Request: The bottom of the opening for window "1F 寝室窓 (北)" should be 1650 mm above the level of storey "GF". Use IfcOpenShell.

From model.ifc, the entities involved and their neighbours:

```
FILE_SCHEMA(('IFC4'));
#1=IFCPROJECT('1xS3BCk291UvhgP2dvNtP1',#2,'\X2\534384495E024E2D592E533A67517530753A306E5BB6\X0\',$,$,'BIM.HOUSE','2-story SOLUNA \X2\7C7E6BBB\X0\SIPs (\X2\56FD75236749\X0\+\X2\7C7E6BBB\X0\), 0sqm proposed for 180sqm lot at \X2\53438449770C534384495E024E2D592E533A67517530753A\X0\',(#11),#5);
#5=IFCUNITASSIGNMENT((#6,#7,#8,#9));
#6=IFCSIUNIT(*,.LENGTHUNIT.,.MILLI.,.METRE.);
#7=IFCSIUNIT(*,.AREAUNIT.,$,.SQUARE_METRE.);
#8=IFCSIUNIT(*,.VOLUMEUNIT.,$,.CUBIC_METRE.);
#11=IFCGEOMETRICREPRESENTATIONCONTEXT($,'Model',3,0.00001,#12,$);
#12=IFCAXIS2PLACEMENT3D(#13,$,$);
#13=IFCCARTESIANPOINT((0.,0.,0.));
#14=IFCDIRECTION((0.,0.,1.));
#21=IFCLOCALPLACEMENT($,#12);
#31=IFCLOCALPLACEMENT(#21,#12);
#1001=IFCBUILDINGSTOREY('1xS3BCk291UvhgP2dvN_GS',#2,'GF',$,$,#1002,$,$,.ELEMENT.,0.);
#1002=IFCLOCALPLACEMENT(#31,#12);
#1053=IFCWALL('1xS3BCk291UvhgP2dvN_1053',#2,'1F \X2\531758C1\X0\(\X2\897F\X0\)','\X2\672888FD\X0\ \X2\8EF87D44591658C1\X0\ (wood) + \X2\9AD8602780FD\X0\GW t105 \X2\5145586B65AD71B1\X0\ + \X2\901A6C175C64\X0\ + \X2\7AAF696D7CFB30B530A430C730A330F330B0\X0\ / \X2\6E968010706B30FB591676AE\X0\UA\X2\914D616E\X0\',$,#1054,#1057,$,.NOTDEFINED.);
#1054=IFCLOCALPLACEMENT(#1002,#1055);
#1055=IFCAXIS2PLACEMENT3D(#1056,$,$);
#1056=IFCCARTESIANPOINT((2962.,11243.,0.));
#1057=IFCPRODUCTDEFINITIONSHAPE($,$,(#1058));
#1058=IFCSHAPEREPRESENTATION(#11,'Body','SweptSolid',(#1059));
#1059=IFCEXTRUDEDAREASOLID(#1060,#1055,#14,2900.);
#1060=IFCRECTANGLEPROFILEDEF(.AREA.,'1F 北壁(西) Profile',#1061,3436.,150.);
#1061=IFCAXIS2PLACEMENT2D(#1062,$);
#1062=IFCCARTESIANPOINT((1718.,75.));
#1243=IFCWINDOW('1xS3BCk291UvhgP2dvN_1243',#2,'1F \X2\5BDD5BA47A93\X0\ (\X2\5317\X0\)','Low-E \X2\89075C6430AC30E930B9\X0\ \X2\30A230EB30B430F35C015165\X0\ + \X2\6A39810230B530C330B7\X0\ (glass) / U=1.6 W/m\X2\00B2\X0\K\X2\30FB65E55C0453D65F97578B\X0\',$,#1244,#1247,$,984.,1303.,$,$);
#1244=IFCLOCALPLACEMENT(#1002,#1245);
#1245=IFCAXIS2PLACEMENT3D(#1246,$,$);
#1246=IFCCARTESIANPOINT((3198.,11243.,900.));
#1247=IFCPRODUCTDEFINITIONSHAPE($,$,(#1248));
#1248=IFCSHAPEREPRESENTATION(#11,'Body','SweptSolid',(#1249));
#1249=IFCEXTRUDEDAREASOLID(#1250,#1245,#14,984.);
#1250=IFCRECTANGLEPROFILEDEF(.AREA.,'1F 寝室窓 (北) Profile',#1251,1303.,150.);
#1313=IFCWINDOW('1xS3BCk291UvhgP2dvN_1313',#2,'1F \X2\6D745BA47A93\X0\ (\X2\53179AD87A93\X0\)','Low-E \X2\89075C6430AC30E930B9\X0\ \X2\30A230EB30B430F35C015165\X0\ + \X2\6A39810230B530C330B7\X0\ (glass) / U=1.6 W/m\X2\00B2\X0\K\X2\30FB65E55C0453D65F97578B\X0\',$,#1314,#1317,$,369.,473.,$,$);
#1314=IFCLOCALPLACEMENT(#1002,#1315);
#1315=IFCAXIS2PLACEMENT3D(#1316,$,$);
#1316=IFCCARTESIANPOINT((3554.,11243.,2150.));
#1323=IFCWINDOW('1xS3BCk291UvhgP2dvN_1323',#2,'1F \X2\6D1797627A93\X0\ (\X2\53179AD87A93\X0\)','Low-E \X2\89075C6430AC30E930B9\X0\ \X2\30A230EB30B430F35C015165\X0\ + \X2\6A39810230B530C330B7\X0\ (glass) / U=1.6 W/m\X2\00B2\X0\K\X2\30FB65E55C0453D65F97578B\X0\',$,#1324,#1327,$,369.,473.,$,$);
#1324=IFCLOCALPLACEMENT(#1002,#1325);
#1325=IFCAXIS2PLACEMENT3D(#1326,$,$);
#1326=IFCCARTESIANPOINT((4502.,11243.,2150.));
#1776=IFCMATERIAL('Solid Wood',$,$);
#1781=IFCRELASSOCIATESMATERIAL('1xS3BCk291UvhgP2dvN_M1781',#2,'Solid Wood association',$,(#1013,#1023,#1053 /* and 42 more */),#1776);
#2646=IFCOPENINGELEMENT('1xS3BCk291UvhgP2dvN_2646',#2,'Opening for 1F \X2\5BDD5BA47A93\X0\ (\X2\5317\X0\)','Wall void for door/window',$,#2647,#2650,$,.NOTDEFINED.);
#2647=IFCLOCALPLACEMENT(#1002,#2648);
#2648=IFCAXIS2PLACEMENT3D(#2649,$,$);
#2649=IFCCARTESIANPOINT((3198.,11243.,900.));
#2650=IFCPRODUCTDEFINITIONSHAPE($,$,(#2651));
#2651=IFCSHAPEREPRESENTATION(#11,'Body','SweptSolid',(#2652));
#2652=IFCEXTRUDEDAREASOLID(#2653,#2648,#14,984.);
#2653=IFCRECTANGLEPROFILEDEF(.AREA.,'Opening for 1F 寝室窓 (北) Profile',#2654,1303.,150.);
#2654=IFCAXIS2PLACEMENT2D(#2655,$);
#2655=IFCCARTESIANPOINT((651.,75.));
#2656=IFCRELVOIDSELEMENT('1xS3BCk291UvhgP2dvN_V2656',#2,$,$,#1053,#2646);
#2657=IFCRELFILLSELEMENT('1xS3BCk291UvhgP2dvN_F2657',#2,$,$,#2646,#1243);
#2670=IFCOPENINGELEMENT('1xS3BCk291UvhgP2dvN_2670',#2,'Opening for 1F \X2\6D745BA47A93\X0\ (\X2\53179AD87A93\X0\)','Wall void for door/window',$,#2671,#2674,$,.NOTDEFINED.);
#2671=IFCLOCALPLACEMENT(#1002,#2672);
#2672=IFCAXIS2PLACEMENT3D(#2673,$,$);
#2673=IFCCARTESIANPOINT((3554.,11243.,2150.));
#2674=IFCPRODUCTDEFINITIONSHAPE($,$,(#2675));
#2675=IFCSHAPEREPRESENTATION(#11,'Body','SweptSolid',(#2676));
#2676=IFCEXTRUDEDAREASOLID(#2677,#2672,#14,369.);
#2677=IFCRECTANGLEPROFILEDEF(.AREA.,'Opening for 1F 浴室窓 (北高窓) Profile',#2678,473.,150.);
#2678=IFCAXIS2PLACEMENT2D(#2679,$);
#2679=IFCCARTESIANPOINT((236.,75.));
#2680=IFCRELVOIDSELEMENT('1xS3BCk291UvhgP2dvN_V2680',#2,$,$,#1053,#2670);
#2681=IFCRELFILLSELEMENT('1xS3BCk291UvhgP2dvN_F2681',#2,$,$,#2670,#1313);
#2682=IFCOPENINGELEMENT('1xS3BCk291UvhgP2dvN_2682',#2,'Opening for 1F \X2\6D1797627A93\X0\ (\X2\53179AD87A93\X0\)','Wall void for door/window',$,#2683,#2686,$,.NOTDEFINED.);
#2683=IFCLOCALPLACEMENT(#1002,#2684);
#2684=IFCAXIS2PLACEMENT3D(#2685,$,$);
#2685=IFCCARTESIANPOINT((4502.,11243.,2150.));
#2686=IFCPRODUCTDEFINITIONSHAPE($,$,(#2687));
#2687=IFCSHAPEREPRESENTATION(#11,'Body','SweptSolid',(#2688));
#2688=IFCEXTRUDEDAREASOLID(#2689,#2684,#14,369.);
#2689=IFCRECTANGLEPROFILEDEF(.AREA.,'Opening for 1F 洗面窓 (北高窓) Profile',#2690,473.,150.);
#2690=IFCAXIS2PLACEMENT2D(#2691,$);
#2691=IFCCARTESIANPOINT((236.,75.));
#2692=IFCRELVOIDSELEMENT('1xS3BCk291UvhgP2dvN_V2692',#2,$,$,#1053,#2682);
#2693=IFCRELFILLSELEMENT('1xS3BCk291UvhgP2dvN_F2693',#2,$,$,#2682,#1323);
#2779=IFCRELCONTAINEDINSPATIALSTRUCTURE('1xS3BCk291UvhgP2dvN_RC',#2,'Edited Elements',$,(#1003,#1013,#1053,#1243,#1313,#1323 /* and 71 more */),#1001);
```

```python
import numpy as np
import ifcopenshell
import ifcopenshell.api.geometry
import ifcopenshell.geom
import ifcopenshell.util.element
import ifcopenshell.util.placement
import ifcopenshell.util.shape
import ifcopenshell.util.unit

model = ifcopenshell.open("model.ifc")
unit_scale = ifcopenshell.util.unit.calculate_unit_scale(model)

window = model.by_guid("1xS3BCk291UvhgP2dvN_1243")
opening = window.FillsVoids[0].RelatingOpeningElement
storey = ifcopenshell.util.element.get_container(window, ifc_class="IfcBuildingStorey")
level = ifcopenshell.util.placement.get_local_placement(storey.ObjectPlacement)[2, 3]

# The opening's origin need not be at the sill, so measure its lowest point.
shape = ifcopenshell.geom.create_shape(ifcopenshell.geom.settings(), opening)
bottom = ifcopenshell.util.shape.get_shape_bottom_elevation(shape, shape.geometry) / unit_scale
dz = level + 1.65 / unit_scale - bottom

shift = np.array([0.0, 0.0, dz])
# The window is not placed relative to its opening, so move both.
for product in (opening, window):
    matrix = ifcopenshell.util.placement.get_local_placement(product.ObjectPlacement)
    matrix[:3, 3] += shift
    ifcopenshell.api.geometry.edit_object_placement(model, product=product, matrix=matrix, is_si=False)

print(f"moved by {dz * unit_scale:+.3f} m")

model.write("model_edited.ifc")
```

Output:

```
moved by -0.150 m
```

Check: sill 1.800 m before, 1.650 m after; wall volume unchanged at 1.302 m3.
